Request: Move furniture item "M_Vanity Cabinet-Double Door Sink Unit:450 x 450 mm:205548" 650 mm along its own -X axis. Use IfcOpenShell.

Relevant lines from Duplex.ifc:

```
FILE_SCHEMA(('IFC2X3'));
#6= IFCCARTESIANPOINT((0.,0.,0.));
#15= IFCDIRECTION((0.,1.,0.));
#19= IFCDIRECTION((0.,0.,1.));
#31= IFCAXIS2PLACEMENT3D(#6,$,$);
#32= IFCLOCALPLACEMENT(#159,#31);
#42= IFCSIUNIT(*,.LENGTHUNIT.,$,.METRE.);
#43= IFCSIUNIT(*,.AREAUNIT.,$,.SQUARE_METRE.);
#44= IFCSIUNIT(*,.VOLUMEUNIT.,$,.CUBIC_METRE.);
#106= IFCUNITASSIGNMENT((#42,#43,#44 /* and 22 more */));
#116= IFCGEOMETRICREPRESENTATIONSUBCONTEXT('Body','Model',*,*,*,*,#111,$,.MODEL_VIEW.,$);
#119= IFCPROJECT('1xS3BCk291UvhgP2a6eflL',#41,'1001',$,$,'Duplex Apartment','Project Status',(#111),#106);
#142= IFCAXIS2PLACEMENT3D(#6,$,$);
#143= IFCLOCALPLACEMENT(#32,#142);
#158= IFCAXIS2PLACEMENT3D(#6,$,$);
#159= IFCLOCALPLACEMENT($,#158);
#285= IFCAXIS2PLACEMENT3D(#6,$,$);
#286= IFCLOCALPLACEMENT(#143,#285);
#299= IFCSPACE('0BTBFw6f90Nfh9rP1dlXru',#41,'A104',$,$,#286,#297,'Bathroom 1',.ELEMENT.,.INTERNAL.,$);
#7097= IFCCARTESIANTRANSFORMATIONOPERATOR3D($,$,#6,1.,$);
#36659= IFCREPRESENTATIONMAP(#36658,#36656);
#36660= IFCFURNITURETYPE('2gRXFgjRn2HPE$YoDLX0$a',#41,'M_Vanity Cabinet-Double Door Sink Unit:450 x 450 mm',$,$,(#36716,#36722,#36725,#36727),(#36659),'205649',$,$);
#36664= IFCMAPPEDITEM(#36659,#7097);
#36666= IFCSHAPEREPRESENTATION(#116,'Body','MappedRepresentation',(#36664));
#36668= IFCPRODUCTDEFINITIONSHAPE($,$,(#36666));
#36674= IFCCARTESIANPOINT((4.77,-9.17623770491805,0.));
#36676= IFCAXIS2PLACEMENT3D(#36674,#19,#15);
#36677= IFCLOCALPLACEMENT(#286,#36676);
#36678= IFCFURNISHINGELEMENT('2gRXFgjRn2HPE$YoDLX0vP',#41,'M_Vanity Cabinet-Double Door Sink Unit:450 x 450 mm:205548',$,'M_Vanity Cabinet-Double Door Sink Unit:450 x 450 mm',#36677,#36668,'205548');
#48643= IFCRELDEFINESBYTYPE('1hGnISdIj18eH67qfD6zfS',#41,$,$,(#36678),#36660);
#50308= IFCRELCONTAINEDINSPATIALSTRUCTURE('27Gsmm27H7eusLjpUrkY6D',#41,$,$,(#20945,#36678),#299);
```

```python
import ifcopenshell
import ifcopenshell.api.geometry
import ifcopenshell.util.placement
import ifcopenshell.util.unit

model = ifcopenshell.open("Duplex.ifc")
unit_scale = ifcopenshell.util.unit.calculate_unit_scale(model)

item = model.by_guid("2gRXFgjRn2HPE$YoDLX0vP")
matrix = ifcopenshell.util.placement.get_local_placement(item.ObjectPlacement)
matrix[:3, 3] -= matrix[:3, 0] * 0.65 / unit_scale
ifcopenshell.api.geometry.edit_object_placement(model, product=item, matrix=matrix, is_si=False)

print(ifcopenshell.util.placement.get_local_placement(item.ObjectPlacement).round(3) + 0.0)

model.write("Duplex_edited.ifc")
```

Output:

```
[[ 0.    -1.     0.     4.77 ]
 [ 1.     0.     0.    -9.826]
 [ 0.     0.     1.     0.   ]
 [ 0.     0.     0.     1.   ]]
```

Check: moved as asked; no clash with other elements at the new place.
